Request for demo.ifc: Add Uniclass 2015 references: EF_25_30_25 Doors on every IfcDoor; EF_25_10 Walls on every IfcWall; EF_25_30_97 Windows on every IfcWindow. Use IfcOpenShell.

First a look at what the model holds.

```python
import ifcopenshell

model = ifcopenshell.open("demo.ifc")
print(model.schema)
print("classifications:", [c.Name for c in model.by_type("IfcClassification")])
for ifc_class in ("IfcDoor", "IfcRoof", "IfcStair", "IfcWall", "IfcWindow"):
    print(ifc_class, len(model.by_type(ifc_class)))
```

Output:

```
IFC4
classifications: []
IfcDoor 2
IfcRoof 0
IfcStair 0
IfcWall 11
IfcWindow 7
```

```python
import ifcopenshell
import ifcopenshell.api.classification

model = ifcopenshell.open("demo.ifc")

system = ifcopenshell.api.classification.add_classification(model, classification="Uniclass 2015")

codes = {
    "IfcDoor": ("EF_25_30_25", "Doors"),
    "IfcWall": ("EF_25_10", "Walls"),
    "IfcWindow": ("EF_25_30_97", "Windows"),
}
for ifc_class, (code, name) in codes.items():
    products = model.by_type(ifc_class)
    ifcopenshell.api.classification.add_reference(
        model, products=products, classification=system, identification=code, name=name
    )
    print(code, len(products))

model.write("demo_v2.ifc")
```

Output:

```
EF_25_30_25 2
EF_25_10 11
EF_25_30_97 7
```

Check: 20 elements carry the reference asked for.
